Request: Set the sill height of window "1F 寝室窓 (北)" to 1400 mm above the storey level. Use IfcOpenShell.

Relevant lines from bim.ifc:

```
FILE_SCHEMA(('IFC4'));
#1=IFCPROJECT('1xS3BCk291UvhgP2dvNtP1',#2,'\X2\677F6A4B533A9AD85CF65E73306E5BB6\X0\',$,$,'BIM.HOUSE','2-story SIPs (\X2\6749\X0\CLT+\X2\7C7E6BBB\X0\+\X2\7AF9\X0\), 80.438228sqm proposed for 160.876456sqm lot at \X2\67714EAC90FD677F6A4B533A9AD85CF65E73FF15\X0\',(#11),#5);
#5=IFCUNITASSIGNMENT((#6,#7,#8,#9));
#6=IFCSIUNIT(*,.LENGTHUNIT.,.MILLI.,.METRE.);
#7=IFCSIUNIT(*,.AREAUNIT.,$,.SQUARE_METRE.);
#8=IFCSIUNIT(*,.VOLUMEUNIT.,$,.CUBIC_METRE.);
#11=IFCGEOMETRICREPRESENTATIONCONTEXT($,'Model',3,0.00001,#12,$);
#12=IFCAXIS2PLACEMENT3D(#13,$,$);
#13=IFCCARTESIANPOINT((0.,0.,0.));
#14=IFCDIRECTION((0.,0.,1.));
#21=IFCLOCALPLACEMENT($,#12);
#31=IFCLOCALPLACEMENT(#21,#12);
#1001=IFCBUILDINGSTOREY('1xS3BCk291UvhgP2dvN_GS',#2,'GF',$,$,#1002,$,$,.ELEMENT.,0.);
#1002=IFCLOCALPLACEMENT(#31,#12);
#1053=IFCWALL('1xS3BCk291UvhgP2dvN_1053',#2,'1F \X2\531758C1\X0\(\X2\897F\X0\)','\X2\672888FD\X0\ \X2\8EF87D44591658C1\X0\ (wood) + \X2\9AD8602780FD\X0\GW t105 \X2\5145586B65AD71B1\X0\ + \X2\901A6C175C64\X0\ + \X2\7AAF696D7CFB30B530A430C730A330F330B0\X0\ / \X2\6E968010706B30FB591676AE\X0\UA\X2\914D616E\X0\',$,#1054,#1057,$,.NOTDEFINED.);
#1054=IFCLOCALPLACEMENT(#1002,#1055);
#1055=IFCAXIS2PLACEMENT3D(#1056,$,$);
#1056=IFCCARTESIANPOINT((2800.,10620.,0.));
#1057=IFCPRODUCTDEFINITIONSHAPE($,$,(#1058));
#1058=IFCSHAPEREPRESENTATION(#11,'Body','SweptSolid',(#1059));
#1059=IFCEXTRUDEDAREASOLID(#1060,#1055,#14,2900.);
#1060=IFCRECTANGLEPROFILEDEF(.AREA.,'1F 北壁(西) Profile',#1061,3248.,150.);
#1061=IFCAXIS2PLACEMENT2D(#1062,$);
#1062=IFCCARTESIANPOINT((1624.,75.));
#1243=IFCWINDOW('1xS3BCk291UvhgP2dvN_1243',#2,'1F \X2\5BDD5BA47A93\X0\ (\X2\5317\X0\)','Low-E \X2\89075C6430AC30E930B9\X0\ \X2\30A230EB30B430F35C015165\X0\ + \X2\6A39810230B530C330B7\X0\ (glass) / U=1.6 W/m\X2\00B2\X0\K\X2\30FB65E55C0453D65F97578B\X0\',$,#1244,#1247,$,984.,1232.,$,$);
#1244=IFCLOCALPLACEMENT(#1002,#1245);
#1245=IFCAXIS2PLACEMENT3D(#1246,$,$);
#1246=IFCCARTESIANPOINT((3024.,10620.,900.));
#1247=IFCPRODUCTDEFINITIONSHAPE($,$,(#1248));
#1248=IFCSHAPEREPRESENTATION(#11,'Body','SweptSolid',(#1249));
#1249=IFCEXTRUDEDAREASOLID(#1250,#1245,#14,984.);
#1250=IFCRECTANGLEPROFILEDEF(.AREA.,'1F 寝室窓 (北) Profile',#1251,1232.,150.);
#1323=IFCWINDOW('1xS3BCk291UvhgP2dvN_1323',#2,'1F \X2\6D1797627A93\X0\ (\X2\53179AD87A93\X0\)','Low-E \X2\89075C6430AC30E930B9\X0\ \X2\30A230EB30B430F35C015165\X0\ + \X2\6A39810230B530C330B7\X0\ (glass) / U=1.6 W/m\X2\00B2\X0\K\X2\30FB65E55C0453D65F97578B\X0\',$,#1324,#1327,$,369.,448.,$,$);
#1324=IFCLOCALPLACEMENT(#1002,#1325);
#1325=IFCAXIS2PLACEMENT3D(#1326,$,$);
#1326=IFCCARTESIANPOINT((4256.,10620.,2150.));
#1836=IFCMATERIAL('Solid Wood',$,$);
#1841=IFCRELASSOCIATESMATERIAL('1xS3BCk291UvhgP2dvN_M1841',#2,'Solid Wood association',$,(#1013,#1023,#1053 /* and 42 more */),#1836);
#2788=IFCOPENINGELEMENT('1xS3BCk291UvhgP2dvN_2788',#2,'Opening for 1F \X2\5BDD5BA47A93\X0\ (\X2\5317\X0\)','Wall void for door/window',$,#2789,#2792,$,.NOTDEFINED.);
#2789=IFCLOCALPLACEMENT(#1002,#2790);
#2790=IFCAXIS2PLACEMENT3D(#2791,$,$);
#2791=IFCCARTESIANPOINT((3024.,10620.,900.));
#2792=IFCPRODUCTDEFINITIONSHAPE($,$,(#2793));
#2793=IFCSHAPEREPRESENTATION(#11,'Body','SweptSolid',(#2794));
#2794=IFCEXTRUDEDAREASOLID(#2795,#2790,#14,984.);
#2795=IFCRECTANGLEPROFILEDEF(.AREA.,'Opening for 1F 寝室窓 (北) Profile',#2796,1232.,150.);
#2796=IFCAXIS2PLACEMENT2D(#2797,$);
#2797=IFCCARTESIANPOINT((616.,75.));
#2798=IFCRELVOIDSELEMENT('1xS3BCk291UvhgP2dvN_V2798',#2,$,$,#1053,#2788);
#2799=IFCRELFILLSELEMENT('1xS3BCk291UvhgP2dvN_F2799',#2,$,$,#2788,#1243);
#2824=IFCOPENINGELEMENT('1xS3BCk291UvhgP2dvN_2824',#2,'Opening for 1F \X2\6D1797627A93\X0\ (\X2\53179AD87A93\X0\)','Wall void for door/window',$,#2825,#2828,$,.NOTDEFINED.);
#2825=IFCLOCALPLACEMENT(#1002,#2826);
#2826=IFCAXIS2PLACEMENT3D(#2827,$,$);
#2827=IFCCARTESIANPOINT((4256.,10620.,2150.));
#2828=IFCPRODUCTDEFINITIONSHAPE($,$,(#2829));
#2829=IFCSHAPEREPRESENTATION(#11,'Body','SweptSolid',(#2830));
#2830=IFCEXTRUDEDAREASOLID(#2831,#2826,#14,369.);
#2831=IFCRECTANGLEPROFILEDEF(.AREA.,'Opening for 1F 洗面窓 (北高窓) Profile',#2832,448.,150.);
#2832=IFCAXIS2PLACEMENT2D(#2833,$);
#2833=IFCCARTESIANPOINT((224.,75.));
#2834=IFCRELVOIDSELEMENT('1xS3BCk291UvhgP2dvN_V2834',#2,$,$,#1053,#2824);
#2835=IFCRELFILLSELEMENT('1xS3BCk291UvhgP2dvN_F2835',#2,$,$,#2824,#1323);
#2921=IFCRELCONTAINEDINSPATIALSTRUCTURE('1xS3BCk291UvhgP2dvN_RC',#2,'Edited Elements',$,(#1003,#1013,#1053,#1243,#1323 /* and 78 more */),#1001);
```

```python
import numpy as np
import ifcopenshell
import ifcopenshell.api.geometry
import ifcopenshell.geom
import ifcopenshell.util.element
import ifcopenshell.util.placement
import ifcopenshell.util.shape
import ifcopenshell.util.unit

model = ifcopenshell.open("bim.ifc")
unit_scale = ifcopenshell.util.unit.calculate_unit_scale(model)

window = model.by_guid("1xS3BCk291UvhgP2dvN_1243")
opening = window.FillsVoids[0].RelatingOpeningElement
storey = ifcopenshell.util.element.get_container(window, ifc_class="IfcBuildingStorey")
level = ifcopenshell.util.placement.get_local_placement(storey.ObjectPlacement)[2, 3]

# The opening's origin need not be at the sill, so measure its lowest point.
shape = ifcopenshell.geom.create_shape(ifcopenshell.geom.settings(), opening)
bottom = ifcopenshell.util.shape.get_shape_bottom_elevation(shape, shape.geometry) / unit_scale
dz = level + 1.4 / unit_scale - bottom

shift = np.array([0.0, 0.0, dz])
# The window is not placed relative to its opening, so move both.
for product in (opening, window):
    matrix = ifcopenshell.util.placement.get_local_placement(product.ObjectPlacement)
    matrix[:3, 3] += shift
    ifcopenshell.api.geometry.edit_object_placement(model, product=product, matrix=matrix, is_si=False)

print(f"moved by {dz * unit_scale:+.3f} m")

model.write("bim_v2.ifc")
```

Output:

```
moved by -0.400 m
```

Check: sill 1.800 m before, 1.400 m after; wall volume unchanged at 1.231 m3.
